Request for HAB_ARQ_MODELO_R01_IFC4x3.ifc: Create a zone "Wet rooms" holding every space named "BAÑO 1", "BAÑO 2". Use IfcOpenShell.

First a look at what the model holds.

```python
import ifcopenshell

model = ifcopenshell.open("HAB_ARQ_MODELO_R01_IFC4x3.ifc")
print(model.schema)
seen = {}
for space in model.by_type("IfcSpace"):
    seen[space.LongName] = seen.get(space.LongName, 0) + 1
for name, count in sorted(seen.items(), key=str):
    print(count, "x", name)
print("zones:", [z.Name for z in model.by_type("IfcZone")][:20])
```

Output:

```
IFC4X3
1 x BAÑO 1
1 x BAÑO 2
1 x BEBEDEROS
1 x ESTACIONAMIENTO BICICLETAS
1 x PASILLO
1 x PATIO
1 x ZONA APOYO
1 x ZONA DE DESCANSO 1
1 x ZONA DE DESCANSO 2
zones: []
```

```python
import ifcopenshell
import ifcopenshell.api.group
import ifcopenshell.api.root

model = ifcopenshell.open("HAB_ARQ_MODELO_R01_IFC4x3.ifc")

names = {"BAÑO 1", "BAÑO 2"}
spaces = [s for s in model.by_type("IfcSpace") if s.LongName in names]

zone = ifcopenshell.api.root.create_entity(model, ifc_class="IfcZone", name="Wet rooms")
ifcopenshell.api.group.assign_group(model, products=spaces, group=zone)
print(len(spaces), "spaces in", zone.Name)

model.write("HAB_ARQ_MODELO_R01_IFC4x3_updated.ifc")
```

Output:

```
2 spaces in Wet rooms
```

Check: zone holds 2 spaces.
